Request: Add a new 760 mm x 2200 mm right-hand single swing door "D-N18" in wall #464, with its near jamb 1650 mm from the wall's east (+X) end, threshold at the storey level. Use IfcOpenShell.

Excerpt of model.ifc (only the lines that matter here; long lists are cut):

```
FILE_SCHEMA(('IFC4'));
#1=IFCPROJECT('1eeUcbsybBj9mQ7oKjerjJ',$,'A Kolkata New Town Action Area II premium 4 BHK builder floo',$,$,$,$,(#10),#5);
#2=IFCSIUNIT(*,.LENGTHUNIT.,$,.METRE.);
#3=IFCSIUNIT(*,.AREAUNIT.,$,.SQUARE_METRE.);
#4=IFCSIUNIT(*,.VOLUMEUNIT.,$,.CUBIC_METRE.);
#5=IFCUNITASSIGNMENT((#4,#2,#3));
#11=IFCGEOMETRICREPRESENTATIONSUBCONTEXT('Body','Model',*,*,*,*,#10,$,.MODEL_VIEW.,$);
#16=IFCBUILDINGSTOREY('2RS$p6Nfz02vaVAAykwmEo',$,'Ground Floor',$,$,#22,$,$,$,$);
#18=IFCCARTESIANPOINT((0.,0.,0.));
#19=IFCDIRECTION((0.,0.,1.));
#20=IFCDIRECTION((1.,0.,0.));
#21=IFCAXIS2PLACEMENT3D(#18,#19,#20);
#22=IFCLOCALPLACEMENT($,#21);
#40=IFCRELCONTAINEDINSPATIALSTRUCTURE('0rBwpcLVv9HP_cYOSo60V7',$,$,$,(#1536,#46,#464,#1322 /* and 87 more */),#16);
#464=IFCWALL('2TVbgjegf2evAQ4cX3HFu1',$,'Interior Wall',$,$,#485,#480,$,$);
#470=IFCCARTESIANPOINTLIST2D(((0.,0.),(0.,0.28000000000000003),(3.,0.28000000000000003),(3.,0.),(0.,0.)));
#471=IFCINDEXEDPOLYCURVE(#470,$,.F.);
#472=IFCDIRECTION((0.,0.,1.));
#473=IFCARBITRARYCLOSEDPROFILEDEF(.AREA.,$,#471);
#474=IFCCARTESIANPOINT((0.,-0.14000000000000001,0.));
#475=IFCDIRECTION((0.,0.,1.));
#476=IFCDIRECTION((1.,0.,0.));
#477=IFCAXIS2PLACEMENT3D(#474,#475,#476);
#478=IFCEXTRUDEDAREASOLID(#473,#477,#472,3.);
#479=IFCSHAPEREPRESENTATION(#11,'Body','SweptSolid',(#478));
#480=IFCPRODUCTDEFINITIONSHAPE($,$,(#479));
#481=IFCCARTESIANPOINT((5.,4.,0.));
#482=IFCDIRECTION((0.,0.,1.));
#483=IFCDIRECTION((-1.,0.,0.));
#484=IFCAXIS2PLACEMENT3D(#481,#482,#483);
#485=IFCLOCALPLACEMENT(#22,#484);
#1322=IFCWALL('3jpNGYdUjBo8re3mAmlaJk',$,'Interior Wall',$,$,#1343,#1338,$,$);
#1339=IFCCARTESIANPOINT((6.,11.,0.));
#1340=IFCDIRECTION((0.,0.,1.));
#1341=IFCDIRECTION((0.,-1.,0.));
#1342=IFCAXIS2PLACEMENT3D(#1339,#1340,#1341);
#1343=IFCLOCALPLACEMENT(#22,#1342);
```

```python
import numpy as np
import ifcopenshell
import ifcopenshell.api.feature
import ifcopenshell.api.geometry
import ifcopenshell.api.root
import ifcopenshell.api.spatial
import ifcopenshell.geom
import ifcopenshell.util.element
import ifcopenshell.util.placement
import ifcopenshell.util.representation
import ifcopenshell.util.shape
import ifcopenshell.util.unit

model = ifcopenshell.open("model.ifc")
unit_scale = ifcopenshell.util.unit.calculate_unit_scale(model)
settings = ifcopenshell.geom.settings()


def volume(element):
    """Net volume in cubic metres, openings subtracted."""
    shape = ifcopenshell.geom.create_shape(settings, element)
    return ifcopenshell.util.shape.get_volume(shape.geometry)


wall = model.by_guid("2TVbgjegf2evAQ4cX3HFu1")
storey = ifcopenshell.util.element.get_container(wall, ifc_class="IfcBuildingStorey")
context = ifcopenshell.util.representation.get_context(model, "Model", "Body", "MODEL_VIEW")
before = volume(wall)

width, height, from_end, sill = 0.76, 2.2, 1.65, 0.0  # metres

# The wall runs along its own X axis, and the end named is its -X end.
wall_shape = ifcopenshell.geom.create_shape(settings, wall)
x, y, z = ifcopenshell.util.shape.get_vertices(wall_shape.geometry).T
start = x.min() + from_end
face, thickness = float(y.min()), float(y.max() - y.min())
wall_matrix = ifcopenshell.util.placement.get_local_placement(wall.ObjectPlacement)
level = ifcopenshell.util.placement.get_local_placement(storey.ObjectPlacement)[2, 3]


def in_wall(x, y):
    """Placement at x, y metres in the wall's axes, at sill height."""
    matrix = wall_matrix.copy()
    matrix[:, 3] = wall_matrix @ np.array([x / unit_scale, y / unit_scale, 0.0, 1.0])
    matrix[2, 3] = level + sill / unit_scale
    return matrix


# Opening: a box that overshoots both wall faces by 50 mm.
opening = ifcopenshell.api.root.create_entity(model, ifc_class="IfcOpeningElement", predefined_type="OPENING")
box = ifcopenshell.api.geometry.add_wall_representation(
    model, context=context, length=width, height=height, thickness=thickness + 0.1
)
ifcopenshell.api.geometry.assign_representation(model, product=opening, representation=box)
ifcopenshell.api.geometry.edit_object_placement(model, product=opening, matrix=in_wall(start, face - 0.05), is_si=False)
ifcopenshell.api.feature.add_feature(model, feature=opening, element=wall)

door = ifcopenshell.api.root.create_entity(model, ifc_class="IfcDoor", name="D-N18", predefined_type="DOOR")
door.OverallWidth, door.OverallHeight = width / unit_scale, height / unit_scale
door.OperationType = "SINGLE_SWING_RIGHT"
body = ifcopenshell.api.geometry.add_door_representation(
    model,
    context=context,
    overall_width=door.OverallWidth,
    overall_height=door.OverallHeight,
    operation_type="SINGLE_SWING_RIGHT",
    lining_properties={"LiningDepth": thickness / unit_scale, "ThresholdDepth": thickness / unit_scale},
)
ifcopenshell.api.geometry.assign_representation(model, product=door, representation=body)
ifcopenshell.api.spatial.assign_container(model, products=[door], relating_structure=storey)
ifcopenshell.api.feature.add_filling(model, opening=opening, element=door)

# The lining spans the wall, so the door starts at the wall face.
ifcopenshell.api.geometry.edit_object_placement(model, product=door, matrix=in_wall(start, face), is_si=False)

after = volume(wall)

print(f"wall volume {before:.3f} -> {after:.3f} m3")

model.write("model_edited.ifc")
```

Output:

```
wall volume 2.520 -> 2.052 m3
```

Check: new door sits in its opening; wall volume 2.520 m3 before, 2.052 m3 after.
